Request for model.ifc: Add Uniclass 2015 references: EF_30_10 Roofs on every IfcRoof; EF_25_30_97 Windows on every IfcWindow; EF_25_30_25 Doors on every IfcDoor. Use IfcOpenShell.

First a look at what the model holds.

```python
import ifcopenshell

model = ifcopenshell.open("model.ifc")
print(model.schema)
print("classifications:", [c.Name for c in model.by_type("IfcClassification")])
for ifc_class in ("IfcDoor", "IfcRoof", "IfcStair", "IfcWall", "IfcWindow"):
    print(ifc_class, len(model.by_type(ifc_class)))
```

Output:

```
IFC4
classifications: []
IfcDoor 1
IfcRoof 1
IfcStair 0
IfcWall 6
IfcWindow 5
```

```python
import ifcopenshell
import ifcopenshell.api.classification

model = ifcopenshell.open("model.ifc")

system = ifcopenshell.api.classification.add_classification(model, classification="Uniclass 2015")

codes = {
    "IfcRoof": ("EF_30_10", "Roofs"),
    "IfcWindow": ("EF_25_30_97", "Windows"),
    "IfcDoor": ("EF_25_30_25", "Doors"),
}
for ifc_class, (code, name) in codes.items():
    products = model.by_type(ifc_class)
    ifcopenshell.api.classification.add_reference(
        model, products=products, classification=system, identification=code, name=name
    )
    print(code, len(products))

model.write("model_updated.ifc")
```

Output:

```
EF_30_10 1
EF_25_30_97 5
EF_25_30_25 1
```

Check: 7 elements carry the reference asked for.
